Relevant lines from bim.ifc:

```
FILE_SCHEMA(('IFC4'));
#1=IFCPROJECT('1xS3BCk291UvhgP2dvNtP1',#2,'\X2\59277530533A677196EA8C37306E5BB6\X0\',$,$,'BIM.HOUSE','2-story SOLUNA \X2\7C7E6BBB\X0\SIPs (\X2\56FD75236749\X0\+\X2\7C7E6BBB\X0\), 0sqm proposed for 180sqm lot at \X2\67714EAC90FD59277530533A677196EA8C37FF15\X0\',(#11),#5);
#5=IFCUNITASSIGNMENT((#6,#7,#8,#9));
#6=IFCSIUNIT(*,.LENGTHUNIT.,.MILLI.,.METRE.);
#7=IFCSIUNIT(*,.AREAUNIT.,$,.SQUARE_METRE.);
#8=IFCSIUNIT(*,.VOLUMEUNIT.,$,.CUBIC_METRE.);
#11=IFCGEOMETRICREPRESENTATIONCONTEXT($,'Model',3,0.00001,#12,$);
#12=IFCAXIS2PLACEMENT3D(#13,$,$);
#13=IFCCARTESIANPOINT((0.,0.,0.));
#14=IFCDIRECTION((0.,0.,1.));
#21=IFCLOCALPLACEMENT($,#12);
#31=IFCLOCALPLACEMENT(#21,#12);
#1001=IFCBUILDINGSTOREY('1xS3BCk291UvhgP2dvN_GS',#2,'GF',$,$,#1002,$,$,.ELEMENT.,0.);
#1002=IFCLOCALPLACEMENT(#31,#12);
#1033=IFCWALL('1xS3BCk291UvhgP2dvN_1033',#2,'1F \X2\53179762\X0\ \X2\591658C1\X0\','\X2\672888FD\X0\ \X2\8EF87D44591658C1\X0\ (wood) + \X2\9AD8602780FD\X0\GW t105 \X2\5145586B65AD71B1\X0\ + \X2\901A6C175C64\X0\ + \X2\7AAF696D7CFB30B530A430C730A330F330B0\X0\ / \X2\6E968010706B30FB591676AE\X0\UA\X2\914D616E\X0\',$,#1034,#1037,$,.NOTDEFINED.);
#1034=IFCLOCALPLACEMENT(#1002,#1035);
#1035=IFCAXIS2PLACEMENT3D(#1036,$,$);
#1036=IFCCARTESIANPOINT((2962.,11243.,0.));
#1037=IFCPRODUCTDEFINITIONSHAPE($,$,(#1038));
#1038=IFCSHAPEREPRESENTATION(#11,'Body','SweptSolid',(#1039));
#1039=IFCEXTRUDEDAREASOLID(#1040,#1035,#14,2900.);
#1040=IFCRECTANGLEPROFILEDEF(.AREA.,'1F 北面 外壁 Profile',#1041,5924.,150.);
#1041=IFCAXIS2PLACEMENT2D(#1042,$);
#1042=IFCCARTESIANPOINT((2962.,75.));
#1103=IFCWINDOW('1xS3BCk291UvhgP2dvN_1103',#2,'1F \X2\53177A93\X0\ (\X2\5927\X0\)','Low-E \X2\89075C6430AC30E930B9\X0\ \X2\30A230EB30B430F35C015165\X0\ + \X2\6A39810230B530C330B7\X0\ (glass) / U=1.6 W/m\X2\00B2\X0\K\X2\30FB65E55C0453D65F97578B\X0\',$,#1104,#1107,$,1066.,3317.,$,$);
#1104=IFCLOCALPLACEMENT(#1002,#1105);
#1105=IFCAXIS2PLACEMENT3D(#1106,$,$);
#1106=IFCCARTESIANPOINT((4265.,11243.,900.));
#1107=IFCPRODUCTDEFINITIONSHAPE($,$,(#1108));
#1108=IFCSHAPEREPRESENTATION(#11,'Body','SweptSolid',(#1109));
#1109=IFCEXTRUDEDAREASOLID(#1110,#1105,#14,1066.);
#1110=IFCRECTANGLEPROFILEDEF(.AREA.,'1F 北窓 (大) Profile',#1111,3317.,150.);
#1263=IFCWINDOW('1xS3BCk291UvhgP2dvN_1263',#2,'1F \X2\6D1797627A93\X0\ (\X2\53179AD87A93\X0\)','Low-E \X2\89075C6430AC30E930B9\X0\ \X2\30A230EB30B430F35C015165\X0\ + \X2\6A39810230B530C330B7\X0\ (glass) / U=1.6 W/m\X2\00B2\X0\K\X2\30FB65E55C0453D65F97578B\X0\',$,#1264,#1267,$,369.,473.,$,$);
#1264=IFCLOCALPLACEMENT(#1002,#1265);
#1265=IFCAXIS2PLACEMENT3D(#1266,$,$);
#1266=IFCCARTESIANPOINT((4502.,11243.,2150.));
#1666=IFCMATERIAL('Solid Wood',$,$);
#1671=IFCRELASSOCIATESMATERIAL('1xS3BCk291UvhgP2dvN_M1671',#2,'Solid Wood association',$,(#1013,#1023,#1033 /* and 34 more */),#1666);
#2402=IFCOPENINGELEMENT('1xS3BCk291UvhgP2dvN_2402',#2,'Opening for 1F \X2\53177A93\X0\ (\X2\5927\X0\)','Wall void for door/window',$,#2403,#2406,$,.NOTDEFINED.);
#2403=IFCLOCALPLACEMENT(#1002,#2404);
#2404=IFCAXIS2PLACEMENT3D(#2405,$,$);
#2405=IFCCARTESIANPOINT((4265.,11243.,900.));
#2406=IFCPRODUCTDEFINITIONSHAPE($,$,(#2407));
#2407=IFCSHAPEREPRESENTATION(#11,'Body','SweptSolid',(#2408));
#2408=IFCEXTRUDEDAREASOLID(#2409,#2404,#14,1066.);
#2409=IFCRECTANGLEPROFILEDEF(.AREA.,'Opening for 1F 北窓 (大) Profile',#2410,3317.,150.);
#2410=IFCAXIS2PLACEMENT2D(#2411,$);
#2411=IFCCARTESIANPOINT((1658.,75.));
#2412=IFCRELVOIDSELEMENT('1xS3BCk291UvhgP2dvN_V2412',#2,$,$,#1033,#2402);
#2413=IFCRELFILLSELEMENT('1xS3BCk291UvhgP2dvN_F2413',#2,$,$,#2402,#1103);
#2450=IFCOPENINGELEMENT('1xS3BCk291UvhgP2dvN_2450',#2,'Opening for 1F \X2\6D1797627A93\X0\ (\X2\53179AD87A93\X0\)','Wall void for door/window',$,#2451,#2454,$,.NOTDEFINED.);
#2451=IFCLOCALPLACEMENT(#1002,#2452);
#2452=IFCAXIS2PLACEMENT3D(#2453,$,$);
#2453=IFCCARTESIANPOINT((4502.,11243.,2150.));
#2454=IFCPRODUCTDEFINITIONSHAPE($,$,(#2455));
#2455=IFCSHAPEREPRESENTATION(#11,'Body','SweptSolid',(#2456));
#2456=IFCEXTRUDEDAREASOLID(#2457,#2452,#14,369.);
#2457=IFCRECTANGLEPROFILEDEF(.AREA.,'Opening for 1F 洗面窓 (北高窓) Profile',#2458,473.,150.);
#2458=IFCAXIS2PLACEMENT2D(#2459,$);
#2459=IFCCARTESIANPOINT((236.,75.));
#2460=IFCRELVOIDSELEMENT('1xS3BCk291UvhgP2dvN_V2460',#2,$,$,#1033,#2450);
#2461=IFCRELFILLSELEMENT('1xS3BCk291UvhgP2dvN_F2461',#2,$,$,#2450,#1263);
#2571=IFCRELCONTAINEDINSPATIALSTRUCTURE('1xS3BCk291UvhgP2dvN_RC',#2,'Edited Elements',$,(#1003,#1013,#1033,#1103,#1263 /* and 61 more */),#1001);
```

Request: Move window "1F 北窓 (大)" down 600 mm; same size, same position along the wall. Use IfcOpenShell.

```python
import numpy as np
import ifcopenshell
import ifcopenshell.api.geometry
import ifcopenshell.util.placement
import ifcopenshell.util.unit

model = ifcopenshell.open("bim.ifc")
unit_scale = ifcopenshell.util.unit.calculate_unit_scale(model)

window = model.by_guid("1xS3BCk291UvhgP2dvN_1103")
opening = window.FillsVoids[0].RelatingOpeningElement
dz = -0.6 / unit_scale

shift = np.array([0.0, 0.0, dz])
# The window is not placed relative to its opening, so move both.
for product in (opening, window):
    matrix = ifcopenshell.util.placement.get_local_placement(product.ObjectPlacement)
    matrix[:3, 3] += shift
    ifcopenshell.api.geometry.edit_object_placement(model, product=product, matrix=matrix, is_si=False)

print(f"moved by {dz * unit_scale:+.3f} m")

model.write("bim_rev.ifc")
```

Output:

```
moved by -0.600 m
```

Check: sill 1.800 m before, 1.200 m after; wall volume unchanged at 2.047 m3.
